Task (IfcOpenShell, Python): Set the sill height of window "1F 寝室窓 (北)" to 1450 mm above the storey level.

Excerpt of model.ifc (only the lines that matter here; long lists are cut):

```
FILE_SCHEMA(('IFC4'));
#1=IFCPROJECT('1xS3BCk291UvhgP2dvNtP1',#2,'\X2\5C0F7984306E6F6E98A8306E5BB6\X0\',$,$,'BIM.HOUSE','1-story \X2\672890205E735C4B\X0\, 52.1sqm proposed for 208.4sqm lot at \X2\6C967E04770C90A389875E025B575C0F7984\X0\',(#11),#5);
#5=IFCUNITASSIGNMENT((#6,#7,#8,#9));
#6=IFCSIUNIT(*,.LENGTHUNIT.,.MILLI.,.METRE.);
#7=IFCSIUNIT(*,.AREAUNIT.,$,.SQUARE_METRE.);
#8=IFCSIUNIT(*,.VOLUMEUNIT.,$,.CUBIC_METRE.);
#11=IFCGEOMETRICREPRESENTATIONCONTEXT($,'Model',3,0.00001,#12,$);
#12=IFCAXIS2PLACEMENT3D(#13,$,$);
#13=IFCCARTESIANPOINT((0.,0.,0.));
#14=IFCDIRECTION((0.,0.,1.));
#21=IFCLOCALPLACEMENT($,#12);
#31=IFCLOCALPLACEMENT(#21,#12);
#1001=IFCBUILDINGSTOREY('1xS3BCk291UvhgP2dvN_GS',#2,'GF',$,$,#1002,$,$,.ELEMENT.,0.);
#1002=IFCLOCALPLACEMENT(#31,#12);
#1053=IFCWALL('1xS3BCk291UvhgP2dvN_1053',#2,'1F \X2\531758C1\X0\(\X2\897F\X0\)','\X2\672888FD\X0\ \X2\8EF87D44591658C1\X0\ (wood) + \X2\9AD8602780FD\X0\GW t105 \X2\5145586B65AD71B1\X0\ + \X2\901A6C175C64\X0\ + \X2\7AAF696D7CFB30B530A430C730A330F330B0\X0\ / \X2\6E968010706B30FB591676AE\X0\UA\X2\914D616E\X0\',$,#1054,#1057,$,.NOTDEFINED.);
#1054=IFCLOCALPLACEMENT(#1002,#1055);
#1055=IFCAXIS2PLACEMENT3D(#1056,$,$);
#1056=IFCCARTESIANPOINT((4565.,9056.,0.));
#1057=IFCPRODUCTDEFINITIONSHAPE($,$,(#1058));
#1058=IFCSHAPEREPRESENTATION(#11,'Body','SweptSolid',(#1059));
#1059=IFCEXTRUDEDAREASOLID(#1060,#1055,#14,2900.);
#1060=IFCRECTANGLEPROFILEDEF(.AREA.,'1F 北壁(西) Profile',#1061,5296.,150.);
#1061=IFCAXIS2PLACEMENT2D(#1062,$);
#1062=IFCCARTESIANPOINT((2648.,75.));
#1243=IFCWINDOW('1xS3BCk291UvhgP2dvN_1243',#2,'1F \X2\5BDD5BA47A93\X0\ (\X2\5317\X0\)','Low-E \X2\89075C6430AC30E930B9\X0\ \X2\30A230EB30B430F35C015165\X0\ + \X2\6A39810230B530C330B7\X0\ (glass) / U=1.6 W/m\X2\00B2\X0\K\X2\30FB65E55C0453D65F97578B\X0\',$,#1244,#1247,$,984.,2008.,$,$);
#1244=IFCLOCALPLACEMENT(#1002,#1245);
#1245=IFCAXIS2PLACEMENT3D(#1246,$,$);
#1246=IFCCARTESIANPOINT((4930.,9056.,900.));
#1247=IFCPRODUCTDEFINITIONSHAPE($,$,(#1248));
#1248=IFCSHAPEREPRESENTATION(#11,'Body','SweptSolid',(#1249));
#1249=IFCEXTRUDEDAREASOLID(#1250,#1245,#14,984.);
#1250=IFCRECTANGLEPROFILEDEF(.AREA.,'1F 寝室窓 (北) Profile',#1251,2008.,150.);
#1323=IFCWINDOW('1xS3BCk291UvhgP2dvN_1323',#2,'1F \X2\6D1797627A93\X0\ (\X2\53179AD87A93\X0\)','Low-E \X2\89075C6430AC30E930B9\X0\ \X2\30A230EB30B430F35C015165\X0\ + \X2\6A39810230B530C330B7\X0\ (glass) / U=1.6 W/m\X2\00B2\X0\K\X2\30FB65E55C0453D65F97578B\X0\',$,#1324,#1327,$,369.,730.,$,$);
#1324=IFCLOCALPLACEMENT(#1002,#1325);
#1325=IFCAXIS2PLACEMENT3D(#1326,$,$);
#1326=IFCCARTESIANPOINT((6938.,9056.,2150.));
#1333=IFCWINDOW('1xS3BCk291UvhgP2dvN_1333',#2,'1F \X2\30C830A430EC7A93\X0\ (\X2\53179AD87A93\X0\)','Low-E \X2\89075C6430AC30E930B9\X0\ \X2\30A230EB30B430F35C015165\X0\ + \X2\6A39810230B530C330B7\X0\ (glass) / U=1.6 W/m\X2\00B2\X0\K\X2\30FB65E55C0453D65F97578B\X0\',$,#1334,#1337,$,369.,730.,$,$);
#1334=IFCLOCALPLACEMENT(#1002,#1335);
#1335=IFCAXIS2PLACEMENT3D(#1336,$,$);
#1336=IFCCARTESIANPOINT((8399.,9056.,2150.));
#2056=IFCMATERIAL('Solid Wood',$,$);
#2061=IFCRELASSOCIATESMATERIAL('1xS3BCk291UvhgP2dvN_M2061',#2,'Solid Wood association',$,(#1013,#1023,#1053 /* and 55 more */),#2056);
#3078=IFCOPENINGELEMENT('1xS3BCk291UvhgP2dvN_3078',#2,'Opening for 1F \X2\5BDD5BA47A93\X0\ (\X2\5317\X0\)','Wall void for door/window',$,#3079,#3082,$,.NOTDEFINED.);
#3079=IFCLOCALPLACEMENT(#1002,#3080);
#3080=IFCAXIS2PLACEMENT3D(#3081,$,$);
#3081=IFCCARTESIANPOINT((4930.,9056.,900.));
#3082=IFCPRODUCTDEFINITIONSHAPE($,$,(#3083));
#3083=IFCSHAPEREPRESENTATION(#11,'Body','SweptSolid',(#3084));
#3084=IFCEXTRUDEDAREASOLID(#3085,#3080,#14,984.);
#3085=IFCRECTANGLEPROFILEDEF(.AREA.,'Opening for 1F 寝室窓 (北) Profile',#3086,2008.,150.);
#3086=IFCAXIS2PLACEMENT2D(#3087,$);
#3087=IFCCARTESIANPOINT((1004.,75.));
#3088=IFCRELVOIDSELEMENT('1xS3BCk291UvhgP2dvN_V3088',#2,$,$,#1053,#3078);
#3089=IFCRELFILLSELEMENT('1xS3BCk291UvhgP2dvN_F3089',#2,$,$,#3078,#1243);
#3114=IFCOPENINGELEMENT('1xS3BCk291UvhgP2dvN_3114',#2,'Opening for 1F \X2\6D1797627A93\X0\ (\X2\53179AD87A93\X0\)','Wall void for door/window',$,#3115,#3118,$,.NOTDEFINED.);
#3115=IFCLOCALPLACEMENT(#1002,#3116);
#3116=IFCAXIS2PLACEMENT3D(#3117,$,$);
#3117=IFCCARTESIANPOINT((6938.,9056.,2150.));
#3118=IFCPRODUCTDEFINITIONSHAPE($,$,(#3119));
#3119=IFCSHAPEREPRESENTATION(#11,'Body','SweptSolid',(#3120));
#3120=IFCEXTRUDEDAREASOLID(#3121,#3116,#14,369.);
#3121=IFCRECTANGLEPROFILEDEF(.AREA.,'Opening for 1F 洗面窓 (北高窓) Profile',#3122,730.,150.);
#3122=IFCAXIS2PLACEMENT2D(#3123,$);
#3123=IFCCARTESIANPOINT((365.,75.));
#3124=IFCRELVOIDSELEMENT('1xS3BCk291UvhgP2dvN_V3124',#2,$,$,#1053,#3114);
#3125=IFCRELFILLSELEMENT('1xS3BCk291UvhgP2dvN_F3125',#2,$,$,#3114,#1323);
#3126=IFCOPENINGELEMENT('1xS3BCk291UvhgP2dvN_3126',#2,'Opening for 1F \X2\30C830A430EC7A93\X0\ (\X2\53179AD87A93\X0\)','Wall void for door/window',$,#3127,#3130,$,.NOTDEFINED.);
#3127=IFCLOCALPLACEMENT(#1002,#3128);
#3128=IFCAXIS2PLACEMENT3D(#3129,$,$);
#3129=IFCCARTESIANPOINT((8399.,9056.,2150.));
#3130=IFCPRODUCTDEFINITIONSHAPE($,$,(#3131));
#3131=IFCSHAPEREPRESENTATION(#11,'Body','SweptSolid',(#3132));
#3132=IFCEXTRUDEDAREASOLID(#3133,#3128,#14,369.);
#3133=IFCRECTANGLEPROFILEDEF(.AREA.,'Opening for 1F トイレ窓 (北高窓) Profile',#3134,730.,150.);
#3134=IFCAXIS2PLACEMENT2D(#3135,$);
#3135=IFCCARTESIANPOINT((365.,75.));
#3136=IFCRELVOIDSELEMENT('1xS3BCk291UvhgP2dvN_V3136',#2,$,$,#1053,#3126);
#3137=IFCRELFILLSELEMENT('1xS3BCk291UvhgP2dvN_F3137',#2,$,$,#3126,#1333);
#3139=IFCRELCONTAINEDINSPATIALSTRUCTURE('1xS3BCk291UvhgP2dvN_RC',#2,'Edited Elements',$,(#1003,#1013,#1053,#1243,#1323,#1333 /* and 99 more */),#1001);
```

```python
import numpy as np
import ifcopenshell
import ifcopenshell.api.geometry
import ifcopenshell.geom
import ifcopenshell.util.element
import ifcopenshell.util.placement
import ifcopenshell.util.shape
import ifcopenshell.util.unit

model = ifcopenshell.open("model.ifc")
unit_scale = ifcopenshell.util.unit.calculate_unit_scale(model)

window = model.by_guid("1xS3BCk291UvhgP2dvN_1243")
opening = window.FillsVoids[0].RelatingOpeningElement
storey = ifcopenshell.util.element.get_container(window, ifc_class="IfcBuildingStorey")
level = ifcopenshell.util.placement.get_local_placement(storey.ObjectPlacement)[2, 3]

# The opening's origin need not be at the sill, so measure its lowest point.
shape = ifcopenshell.geom.create_shape(ifcopenshell.geom.settings(), opening)
bottom = ifcopenshell.util.shape.get_shape_bottom_elevation(shape, shape.geometry) / unit_scale
dz = level + 1.45 / unit_scale - bottom

shift = np.array([0.0, 0.0, dz])
# The window is not placed relative to its opening, so move both.
for product in (opening, window):
    matrix = ifcopenshell.util.placement.get_local_placement(product.ObjectPlacement)
    matrix[:3, 3] += shift
    ifcopenshell.api.geometry.edit_object_placement(model, product=product, matrix=matrix, is_si=False)

print(f"moved by {dz * unit_scale:+.3f} m")

model.write("model-out.ifc")
```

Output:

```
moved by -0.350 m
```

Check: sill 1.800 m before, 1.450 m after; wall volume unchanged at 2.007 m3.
